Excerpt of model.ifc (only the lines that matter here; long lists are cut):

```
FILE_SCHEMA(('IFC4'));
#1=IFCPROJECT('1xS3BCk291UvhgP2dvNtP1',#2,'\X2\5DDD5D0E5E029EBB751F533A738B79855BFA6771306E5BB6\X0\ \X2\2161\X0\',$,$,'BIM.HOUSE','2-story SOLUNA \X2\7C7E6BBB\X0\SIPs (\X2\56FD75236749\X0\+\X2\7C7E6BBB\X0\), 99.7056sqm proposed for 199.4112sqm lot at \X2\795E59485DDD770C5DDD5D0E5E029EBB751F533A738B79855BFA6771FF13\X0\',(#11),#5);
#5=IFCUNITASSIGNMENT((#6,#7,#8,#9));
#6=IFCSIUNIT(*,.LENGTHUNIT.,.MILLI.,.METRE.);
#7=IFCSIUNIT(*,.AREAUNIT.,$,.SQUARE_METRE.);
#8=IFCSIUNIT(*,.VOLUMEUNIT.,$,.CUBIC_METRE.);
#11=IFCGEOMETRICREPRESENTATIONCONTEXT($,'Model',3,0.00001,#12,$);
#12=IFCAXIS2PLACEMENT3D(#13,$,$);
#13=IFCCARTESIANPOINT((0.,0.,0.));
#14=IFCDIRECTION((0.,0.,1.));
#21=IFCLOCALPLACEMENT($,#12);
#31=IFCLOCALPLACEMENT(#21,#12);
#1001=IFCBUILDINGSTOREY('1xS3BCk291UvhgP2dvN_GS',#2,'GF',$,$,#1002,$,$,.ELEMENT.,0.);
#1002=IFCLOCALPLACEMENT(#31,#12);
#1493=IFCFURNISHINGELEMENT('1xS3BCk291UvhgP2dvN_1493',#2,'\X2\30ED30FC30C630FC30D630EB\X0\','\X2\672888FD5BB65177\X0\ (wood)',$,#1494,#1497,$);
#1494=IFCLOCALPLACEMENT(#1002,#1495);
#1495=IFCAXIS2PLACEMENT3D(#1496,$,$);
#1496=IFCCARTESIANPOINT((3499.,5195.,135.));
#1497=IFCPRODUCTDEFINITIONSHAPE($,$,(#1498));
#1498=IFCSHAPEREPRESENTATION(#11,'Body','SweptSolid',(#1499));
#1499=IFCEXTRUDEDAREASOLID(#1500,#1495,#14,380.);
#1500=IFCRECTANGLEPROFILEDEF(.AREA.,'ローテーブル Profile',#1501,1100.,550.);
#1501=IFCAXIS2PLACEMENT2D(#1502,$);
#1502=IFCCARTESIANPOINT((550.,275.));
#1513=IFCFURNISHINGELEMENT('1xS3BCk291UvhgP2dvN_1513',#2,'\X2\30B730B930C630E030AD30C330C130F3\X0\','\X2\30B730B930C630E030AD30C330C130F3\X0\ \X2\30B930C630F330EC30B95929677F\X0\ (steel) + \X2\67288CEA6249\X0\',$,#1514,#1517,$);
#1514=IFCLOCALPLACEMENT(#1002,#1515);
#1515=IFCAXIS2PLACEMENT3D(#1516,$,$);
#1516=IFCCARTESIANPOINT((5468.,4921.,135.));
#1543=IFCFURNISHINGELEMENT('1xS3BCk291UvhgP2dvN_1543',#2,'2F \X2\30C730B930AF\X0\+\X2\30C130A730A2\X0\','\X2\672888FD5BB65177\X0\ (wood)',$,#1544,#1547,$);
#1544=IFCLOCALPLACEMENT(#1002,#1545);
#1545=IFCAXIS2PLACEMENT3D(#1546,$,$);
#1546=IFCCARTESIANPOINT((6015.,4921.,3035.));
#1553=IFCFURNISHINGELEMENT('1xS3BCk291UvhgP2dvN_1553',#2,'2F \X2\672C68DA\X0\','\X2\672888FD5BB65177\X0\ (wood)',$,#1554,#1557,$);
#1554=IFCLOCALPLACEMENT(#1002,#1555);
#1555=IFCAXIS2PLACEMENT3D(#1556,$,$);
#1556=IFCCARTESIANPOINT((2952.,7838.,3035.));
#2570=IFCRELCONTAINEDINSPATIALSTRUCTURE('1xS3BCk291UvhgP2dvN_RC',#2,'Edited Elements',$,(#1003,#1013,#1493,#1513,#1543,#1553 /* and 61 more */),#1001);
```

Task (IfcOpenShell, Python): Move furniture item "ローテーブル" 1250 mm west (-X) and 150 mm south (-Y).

```python
import ifcopenshell
import ifcopenshell.api.geometry
import ifcopenshell.util.placement
import ifcopenshell.util.unit

model = ifcopenshell.open("model.ifc")
unit_scale = ifcopenshell.util.unit.calculate_unit_scale(model)

item = model.by_guid("1xS3BCk291UvhgP2dvN_1493")
matrix = ifcopenshell.util.placement.get_local_placement(item.ObjectPlacement)
matrix[0, 3] -= 1.25 / unit_scale
matrix[1, 3] -= 0.15 / unit_scale
ifcopenshell.api.geometry.edit_object_placement(model, product=item, matrix=matrix, is_si=False)

print(ifcopenshell.util.placement.get_local_placement(item.ObjectPlacement).round(3) + 0.0)

model.write("model_updated.ifc")
```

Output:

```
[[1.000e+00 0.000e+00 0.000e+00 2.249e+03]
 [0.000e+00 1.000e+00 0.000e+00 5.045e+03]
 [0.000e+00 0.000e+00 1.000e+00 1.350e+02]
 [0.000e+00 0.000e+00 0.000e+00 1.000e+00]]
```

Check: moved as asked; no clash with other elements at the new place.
